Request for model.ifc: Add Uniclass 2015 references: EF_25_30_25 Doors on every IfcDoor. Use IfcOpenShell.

First a look at what the model holds.

```python
import ifcopenshell

model = ifcopenshell.open("model.ifc")
print(model.schema)
print("classifications:", [c.Name for c in model.by_type("IfcClassification")])
for ifc_class in ("IfcDoor", "IfcRoof", "IfcStair", "IfcWall", "IfcWindow"):
    print(ifc_class, len(model.by_type(ifc_class)))
```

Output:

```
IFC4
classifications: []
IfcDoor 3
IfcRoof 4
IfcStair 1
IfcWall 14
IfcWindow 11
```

```python
import ifcopenshell
import ifcopenshell.api.classification

model = ifcopenshell.open("model.ifc")

system = ifcopenshell.api.classification.add_classification(model, classification="Uniclass 2015")

codes = {
    "IfcDoor": ("EF_25_30_25", "Doors"),
}
for ifc_class, (code, name) in codes.items():
    products = model.by_type(ifc_class)
    ifcopenshell.api.classification.add_reference(
        model, products=products, classification=system, identification=code, name=name
    )
    print(code, len(products))

model.write("model_rev.ifc")
```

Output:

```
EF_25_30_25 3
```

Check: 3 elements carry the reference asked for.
